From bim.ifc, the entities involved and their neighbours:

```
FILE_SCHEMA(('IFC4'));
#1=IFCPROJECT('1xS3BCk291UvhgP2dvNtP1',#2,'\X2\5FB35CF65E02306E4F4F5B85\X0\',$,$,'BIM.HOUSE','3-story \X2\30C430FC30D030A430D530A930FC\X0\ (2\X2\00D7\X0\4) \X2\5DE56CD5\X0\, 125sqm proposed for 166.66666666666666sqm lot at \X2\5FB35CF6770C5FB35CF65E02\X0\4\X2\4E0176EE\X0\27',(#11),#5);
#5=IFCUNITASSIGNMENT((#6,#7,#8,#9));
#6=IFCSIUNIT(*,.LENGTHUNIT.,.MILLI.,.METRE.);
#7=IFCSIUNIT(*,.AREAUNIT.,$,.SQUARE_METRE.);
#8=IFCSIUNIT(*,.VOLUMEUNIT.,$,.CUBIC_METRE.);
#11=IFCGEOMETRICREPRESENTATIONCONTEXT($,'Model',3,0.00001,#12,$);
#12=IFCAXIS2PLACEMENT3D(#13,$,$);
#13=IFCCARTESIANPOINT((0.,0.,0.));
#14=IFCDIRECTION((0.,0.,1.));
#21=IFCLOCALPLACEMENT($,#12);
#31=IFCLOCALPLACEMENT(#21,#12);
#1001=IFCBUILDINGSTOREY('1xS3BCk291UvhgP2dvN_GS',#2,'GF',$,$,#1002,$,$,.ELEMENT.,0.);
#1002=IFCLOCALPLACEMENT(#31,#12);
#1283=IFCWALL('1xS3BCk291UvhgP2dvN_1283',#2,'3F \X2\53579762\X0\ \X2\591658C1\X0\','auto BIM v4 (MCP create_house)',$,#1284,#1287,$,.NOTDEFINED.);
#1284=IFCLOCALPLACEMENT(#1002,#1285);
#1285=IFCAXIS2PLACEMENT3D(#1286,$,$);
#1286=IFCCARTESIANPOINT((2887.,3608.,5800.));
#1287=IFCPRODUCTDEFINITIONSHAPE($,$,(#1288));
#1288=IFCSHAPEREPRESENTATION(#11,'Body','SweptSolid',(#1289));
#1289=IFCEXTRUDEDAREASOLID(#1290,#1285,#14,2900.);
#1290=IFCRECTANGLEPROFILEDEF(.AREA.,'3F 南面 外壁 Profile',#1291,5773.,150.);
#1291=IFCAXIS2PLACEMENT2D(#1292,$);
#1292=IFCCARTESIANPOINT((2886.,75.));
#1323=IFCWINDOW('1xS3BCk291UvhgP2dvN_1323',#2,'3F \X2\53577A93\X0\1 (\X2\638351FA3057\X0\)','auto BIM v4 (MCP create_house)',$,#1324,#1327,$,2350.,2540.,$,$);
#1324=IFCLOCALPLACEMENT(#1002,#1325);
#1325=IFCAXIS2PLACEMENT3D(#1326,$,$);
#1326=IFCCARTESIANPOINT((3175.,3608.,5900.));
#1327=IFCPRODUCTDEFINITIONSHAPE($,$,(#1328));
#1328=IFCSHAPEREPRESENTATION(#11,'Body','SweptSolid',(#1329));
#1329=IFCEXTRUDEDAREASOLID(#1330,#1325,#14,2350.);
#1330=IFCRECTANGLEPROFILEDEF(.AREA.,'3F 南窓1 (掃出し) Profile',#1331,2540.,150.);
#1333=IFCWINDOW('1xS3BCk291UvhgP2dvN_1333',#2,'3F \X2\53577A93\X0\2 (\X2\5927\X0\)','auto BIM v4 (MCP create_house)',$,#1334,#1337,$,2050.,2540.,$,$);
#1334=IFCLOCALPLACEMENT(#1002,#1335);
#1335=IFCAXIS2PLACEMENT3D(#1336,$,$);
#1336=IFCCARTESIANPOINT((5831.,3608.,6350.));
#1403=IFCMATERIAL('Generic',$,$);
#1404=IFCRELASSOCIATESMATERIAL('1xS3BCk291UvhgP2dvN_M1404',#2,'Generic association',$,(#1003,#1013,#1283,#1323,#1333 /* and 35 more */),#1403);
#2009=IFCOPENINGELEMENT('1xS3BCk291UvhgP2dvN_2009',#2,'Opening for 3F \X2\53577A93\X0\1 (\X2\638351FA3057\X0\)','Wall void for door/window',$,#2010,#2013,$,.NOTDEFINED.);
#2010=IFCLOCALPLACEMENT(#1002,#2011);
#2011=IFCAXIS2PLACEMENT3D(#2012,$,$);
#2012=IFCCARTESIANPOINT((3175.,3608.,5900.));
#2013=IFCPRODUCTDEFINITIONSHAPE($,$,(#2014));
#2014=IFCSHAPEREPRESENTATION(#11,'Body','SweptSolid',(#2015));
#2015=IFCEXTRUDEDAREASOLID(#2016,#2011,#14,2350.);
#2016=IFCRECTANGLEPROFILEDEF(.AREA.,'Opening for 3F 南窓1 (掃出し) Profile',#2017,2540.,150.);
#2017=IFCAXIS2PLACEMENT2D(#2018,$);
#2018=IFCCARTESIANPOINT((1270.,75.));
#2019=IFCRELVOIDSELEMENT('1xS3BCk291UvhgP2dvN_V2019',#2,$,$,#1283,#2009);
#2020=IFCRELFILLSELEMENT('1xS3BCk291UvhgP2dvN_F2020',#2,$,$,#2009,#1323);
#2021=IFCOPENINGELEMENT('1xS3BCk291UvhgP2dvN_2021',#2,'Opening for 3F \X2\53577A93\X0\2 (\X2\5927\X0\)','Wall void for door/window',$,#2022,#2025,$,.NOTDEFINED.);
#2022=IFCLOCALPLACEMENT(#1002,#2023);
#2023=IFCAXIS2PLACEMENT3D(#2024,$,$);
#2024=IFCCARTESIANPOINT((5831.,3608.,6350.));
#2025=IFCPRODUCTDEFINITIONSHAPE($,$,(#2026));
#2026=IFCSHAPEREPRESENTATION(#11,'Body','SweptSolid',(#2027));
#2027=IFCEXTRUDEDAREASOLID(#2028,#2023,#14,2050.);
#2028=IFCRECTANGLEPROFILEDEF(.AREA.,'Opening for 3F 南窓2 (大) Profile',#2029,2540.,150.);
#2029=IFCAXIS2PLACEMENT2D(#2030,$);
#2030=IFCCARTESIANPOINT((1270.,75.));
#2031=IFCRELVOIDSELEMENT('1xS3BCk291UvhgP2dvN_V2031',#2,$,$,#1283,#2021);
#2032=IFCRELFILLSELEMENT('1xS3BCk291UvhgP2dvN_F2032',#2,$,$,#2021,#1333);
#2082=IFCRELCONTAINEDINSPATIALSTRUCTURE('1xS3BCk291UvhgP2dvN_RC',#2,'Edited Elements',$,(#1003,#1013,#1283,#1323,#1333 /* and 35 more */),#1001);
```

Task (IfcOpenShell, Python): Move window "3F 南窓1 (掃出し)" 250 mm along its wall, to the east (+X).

```python
import ifcopenshell
import ifcopenshell.api.geometry
import ifcopenshell.util.placement
import ifcopenshell.util.unit

model = ifcopenshell.open("bim.ifc")
unit_scale = ifcopenshell.util.unit.calculate_unit_scale(model)

window = model.by_guid("1xS3BCk291UvhgP2dvN_1323")
opening = window.FillsVoids[0].RelatingOpeningElement
wall = opening.VoidsElements[0].RelatingBuildingElement

wall_matrix = ifcopenshell.util.placement.get_local_placement(wall.ObjectPlacement)
shift = wall_matrix[:3, 0] * 0.25 / unit_scale
before = ifcopenshell.util.placement.get_local_placement(window.ObjectPlacement)[:3, 3].copy()

# The window is not placed relative to its opening, so move both.
for product in (opening, window):
    matrix = ifcopenshell.util.placement.get_local_placement(product.ObjectPlacement)
    matrix[:3, 3] += shift
    ifcopenshell.api.geometry.edit_object_placement(model, product=product, matrix=matrix, is_si=False)

after = ifcopenshell.util.placement.get_local_placement(window.ObjectPlacement)[:3, 3]
print("window moved by", (after - before).round(3) + 0.0)

model.write("bim_updated.ifc")
```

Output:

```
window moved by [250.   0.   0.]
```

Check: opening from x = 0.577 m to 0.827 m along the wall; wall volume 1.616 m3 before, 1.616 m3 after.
